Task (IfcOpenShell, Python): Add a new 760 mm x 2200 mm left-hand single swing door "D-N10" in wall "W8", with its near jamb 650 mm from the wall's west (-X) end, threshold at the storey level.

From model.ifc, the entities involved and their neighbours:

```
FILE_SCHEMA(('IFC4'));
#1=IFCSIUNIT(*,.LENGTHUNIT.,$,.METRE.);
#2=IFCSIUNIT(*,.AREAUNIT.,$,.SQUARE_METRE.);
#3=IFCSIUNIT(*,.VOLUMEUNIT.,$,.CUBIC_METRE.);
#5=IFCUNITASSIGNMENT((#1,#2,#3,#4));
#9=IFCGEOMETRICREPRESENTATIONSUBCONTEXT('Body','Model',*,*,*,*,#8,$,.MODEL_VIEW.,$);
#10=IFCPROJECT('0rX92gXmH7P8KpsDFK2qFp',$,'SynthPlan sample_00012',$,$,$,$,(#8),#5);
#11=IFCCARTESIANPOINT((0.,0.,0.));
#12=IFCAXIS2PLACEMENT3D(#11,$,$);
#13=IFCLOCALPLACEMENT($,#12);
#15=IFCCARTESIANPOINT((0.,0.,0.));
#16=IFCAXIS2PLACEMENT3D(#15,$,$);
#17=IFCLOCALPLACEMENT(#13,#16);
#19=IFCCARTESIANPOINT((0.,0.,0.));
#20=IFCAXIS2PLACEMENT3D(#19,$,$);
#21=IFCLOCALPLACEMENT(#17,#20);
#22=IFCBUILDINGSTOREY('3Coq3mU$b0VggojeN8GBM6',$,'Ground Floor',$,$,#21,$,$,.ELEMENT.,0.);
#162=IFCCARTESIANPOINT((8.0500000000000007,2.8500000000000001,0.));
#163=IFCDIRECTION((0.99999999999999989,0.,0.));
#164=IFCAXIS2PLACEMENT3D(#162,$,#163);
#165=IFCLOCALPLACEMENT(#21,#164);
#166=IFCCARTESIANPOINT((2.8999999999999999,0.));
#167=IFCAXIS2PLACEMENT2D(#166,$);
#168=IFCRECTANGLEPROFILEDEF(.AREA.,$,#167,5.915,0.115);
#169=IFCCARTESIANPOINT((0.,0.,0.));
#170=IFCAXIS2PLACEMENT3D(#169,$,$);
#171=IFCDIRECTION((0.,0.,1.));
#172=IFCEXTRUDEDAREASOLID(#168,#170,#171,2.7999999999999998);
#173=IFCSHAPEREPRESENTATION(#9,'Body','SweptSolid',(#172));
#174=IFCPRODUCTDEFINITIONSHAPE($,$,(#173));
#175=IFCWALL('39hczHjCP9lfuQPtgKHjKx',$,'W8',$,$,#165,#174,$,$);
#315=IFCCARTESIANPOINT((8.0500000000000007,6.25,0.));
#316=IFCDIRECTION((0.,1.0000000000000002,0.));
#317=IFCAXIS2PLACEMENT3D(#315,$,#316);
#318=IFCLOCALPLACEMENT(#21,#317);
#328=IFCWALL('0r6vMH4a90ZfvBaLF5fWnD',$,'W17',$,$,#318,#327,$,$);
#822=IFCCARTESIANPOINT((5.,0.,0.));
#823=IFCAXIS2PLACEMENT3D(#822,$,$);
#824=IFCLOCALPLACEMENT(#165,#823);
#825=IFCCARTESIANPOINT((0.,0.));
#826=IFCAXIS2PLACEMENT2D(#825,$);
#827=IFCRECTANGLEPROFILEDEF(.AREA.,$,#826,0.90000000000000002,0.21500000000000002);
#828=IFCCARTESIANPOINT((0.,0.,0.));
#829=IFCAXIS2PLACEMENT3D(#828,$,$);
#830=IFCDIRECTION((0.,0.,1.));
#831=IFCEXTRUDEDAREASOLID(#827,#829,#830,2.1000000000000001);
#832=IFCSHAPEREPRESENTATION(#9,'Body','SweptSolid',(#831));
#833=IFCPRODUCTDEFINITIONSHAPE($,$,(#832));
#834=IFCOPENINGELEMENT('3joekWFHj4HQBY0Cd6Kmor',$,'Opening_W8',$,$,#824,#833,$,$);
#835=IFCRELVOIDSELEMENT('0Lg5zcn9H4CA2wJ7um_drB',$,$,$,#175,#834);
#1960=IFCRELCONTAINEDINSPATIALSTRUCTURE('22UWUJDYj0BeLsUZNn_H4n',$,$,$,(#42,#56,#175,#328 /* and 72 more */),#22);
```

```python
import numpy as np
import ifcopenshell
import ifcopenshell.api.feature
import ifcopenshell.api.geometry
import ifcopenshell.api.root
import ifcopenshell.api.spatial
import ifcopenshell.geom
import ifcopenshell.util.element
import ifcopenshell.util.placement
import ifcopenshell.util.representation
import ifcopenshell.util.shape
import ifcopenshell.util.unit

model = ifcopenshell.open("model.ifc")
unit_scale = ifcopenshell.util.unit.calculate_unit_scale(model)
settings = ifcopenshell.geom.settings()


def volume(element):
    """Net volume in cubic metres, openings subtracted."""
    shape = ifcopenshell.geom.create_shape(settings, element)
    return ifcopenshell.util.shape.get_volume(shape.geometry)


wall = model.by_guid("39hczHjCP9lfuQPtgKHjKx")
storey = ifcopenshell.util.element.get_container(wall, ifc_class="IfcBuildingStorey")
context = ifcopenshell.util.representation.get_context(model, "Model", "Body", "MODEL_VIEW")
before = volume(wall)

width, height, from_end, sill = 0.76, 2.2, 0.65, 0.0  # metres

# The wall runs along its own X axis, and the end named is its -X end.
wall_shape = ifcopenshell.geom.create_shape(settings, wall)
x, y, z = ifcopenshell.util.shape.get_vertices(wall_shape.geometry).T
start = x.min() + from_end
face, thickness = float(y.min()), float(y.max() - y.min())
wall_matrix = ifcopenshell.util.placement.get_local_placement(wall.ObjectPlacement)
level = ifcopenshell.util.placement.get_local_placement(storey.ObjectPlacement)[2, 3]


def in_wall(x, y):
    """Placement at x, y metres in the wall's axes, at sill height."""
    matrix = wall_matrix.copy()
    matrix[:, 3] = wall_matrix @ np.array([x / unit_scale, y / unit_scale, 0.0, 1.0])
    matrix[2, 3] = level + sill / unit_scale
    return matrix


# Opening: a box that overshoots both wall faces by 50 mm.
opening = ifcopenshell.api.root.create_entity(model, ifc_class="IfcOpeningElement", predefined_type="OPENING")
box = ifcopenshell.api.geometry.add_wall_representation(
    model, context=context, length=width, height=height, thickness=thickness + 0.1
)
ifcopenshell.api.geometry.assign_representation(model, product=opening, representation=box)
ifcopenshell.api.geometry.edit_object_placement(model, product=opening, matrix=in_wall(start, face - 0.05), is_si=False)
ifcopenshell.api.feature.add_feature(model, feature=opening, element=wall)

door = ifcopenshell.api.root.create_entity(model, ifc_class="IfcDoor", name="D-N10", predefined_type="DOOR")
door.OverallWidth, door.OverallHeight = width / unit_scale, height / unit_scale
door.OperationType = "SINGLE_SWING_LEFT"
body = ifcopenshell.api.geometry.add_door_representation(
    model,
    context=context,
    overall_width=door.OverallWidth,
    overall_height=door.OverallHeight,
    operation_type="SINGLE_SWING_LEFT",
    lining_properties={"LiningDepth": thickness / unit_scale, "ThresholdDepth": thickness / unit_scale},
)
ifcopenshell.api.geometry.assign_representation(model, product=door, representation=body)
ifcopenshell.api.spatial.assign_container(model, products=[door], relating_structure=storey)
ifcopenshell.api.feature.add_filling(model, opening=opening, element=door)

# The lining spans the wall, so the door starts at the wall face.
ifcopenshell.api.geometry.edit_object_placement(model, product=door, matrix=in_wall(start, face), is_si=False)

after = volume(wall)

print(f"wall volume {before:.3f} -> {after:.3f} m3")

model.write("model_edited.ifc")
```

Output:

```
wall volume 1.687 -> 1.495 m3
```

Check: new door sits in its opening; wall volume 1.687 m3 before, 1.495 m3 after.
